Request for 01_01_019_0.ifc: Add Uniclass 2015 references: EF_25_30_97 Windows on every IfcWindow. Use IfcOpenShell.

First a look at what the model holds.

```python
import ifcopenshell

model = ifcopenshell.open("01_01_019_0.ifc")
print(model.schema)
print("classifications:", [c.Name for c in model.by_type("IfcClassification")])
for ifc_class in ("IfcDoor", "IfcRoof", "IfcStair", "IfcWall", "IfcWindow"):
    print(ifc_class, len(model.by_type(ifc_class)))
```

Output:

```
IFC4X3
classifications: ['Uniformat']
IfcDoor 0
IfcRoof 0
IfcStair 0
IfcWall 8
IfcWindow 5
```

```python
import ifcopenshell
import ifcopenshell.api.classification

model = ifcopenshell.open("01_01_019_0.ifc")

system = ifcopenshell.api.classification.add_classification(model, classification="Uniclass 2015")

codes = {
    "IfcWindow": ("EF_25_30_97", "Windows"),
}
for ifc_class, (code, name) in codes.items():
    products = model.by_type(ifc_class)
    ifcopenshell.api.classification.add_reference(
        model, products=products, classification=system, identification=code, name=name
    )
    print(code, len(products))

model.write("01_01_019_0_rev.ifc")
```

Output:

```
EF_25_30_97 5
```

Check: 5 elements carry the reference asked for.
